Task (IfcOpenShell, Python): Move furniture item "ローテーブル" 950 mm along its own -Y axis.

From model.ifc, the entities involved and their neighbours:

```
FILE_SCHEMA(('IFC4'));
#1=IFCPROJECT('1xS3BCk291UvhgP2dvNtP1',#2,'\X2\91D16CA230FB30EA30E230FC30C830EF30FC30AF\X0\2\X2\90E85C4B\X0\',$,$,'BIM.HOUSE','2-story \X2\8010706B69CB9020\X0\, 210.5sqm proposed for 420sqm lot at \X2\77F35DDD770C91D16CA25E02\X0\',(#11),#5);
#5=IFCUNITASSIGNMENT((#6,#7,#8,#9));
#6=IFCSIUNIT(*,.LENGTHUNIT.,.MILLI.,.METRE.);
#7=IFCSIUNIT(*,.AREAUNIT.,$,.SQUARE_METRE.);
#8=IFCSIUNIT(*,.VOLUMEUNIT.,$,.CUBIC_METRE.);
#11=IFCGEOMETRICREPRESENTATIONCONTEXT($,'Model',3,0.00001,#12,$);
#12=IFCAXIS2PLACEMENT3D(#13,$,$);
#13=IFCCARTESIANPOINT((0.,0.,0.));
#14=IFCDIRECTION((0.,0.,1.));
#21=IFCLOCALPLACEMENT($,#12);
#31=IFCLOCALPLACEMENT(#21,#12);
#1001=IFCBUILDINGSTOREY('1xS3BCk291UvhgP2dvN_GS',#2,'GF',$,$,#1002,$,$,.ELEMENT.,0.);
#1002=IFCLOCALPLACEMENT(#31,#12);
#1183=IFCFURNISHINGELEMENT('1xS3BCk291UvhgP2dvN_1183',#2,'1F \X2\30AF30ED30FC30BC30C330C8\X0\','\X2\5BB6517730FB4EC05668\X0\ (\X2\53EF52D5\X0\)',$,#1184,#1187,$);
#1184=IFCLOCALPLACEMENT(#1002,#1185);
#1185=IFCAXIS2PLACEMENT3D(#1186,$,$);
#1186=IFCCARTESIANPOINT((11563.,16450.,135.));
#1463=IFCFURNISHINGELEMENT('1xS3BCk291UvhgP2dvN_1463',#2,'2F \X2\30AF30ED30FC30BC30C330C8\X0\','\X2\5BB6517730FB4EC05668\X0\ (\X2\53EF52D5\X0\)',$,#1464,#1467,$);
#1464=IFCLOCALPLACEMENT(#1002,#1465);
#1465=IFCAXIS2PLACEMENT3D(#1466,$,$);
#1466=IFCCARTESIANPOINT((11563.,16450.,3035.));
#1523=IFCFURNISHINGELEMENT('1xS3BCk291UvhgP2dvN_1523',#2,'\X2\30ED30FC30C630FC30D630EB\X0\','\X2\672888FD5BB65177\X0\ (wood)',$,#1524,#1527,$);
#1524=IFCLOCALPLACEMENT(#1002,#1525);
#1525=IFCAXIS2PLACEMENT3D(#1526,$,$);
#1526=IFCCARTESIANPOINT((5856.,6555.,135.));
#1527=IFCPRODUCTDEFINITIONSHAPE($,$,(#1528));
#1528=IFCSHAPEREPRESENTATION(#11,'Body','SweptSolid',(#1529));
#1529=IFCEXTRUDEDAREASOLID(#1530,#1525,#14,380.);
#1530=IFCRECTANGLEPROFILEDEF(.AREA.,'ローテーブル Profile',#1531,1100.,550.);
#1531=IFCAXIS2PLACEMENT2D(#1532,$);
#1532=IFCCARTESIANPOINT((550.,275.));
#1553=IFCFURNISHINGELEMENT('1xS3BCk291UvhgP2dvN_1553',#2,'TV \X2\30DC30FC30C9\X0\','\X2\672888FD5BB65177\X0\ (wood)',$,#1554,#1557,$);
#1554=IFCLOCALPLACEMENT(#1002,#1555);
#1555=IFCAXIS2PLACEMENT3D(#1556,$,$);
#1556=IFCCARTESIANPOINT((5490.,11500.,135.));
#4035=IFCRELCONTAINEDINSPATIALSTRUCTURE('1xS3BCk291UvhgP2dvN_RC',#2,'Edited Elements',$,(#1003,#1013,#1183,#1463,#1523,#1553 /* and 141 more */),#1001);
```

```python
import ifcopenshell
import ifcopenshell.api.geometry
import ifcopenshell.util.placement

model = ifcopenshell.open("model.ifc")

item = model.by_guid("1xS3BCk291UvhgP2dvN_1523")
matrix = ifcopenshell.util.placement.get_local_placement(item.ObjectPlacement)
matrix[:3, 3] -= matrix[:3, 1] * 950.0
ifcopenshell.api.geometry.edit_object_placement(model, product=item, matrix=matrix, is_si=False)

print(ifcopenshell.util.placement.get_local_placement(item.ObjectPlacement).round(3) + 0.0)

model.write("model-out.ifc")
```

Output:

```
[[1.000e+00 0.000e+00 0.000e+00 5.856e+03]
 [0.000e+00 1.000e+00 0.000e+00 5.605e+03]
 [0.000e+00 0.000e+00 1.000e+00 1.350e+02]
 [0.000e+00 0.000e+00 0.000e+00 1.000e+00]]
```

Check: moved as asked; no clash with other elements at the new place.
